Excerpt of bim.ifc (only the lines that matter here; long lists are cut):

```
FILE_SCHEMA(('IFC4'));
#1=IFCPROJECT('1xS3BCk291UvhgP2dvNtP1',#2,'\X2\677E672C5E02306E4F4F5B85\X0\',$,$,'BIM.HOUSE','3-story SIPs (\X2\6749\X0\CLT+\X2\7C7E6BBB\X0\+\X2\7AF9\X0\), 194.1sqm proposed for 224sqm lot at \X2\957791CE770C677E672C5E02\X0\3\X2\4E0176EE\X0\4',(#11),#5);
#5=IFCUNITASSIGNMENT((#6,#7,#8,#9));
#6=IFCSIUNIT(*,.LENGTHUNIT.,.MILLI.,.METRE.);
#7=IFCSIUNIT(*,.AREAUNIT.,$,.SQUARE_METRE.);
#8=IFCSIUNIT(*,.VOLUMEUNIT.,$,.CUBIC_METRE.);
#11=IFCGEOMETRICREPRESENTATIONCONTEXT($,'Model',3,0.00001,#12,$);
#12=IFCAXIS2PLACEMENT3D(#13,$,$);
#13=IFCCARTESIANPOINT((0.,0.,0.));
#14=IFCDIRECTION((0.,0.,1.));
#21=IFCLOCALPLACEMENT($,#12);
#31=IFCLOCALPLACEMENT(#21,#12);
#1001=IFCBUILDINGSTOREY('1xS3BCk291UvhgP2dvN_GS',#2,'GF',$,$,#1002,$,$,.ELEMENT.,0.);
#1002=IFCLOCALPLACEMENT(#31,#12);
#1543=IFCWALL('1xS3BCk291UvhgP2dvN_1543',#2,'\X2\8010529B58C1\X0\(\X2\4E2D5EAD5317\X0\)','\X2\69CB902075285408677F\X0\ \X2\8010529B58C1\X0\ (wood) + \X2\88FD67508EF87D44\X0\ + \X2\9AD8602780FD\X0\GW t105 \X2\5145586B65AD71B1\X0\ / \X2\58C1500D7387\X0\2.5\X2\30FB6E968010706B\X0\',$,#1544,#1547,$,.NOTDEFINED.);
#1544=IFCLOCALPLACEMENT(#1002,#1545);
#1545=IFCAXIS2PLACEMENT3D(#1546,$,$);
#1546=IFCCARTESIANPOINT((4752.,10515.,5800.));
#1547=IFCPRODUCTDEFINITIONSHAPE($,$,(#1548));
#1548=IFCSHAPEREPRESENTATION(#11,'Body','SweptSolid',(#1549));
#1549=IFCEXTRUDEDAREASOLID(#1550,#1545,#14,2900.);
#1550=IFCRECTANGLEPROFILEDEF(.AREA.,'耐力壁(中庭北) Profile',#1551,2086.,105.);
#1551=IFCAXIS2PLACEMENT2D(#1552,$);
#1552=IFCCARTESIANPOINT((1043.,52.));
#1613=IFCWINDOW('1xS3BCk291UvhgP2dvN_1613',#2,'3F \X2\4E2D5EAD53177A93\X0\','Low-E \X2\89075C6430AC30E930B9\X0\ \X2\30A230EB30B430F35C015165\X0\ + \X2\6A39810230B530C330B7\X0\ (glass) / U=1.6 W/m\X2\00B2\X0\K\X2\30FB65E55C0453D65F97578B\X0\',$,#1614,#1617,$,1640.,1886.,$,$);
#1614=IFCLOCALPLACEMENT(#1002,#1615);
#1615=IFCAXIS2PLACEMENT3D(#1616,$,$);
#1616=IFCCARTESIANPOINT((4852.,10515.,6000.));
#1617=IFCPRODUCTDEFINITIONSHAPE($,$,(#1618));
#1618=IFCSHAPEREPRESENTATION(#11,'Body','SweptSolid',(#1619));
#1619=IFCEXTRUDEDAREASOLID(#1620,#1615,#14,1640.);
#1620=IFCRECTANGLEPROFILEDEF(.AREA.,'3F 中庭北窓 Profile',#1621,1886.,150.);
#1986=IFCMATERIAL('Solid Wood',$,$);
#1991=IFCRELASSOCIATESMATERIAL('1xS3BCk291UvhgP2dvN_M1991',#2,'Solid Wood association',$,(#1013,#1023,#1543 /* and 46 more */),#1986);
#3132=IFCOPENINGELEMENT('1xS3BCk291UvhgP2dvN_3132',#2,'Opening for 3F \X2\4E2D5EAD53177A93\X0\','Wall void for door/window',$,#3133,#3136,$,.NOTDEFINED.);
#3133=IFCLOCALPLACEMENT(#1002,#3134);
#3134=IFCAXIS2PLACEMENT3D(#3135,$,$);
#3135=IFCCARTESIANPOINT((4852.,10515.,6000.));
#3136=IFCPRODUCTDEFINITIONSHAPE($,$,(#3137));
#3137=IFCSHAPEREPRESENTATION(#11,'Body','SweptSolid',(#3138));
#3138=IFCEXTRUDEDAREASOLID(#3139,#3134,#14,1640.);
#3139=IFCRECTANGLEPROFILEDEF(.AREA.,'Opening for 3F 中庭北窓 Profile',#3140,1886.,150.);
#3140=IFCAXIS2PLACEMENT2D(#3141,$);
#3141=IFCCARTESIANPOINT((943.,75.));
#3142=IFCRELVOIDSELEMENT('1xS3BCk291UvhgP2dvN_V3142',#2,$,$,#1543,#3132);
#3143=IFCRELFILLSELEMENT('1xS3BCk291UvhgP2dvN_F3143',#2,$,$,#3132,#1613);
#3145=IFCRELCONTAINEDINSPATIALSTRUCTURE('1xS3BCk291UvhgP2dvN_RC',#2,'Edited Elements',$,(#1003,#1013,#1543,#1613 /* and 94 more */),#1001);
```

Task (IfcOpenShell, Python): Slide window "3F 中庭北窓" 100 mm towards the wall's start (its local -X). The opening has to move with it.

```python
import ifcopenshell
import ifcopenshell.api.geometry
import ifcopenshell.util.placement

model = ifcopenshell.open("bim.ifc")

window = model.by_guid("1xS3BCk291UvhgP2dvN_1613")
opening = window.FillsVoids[0].RelatingOpeningElement
wall = opening.VoidsElements[0].RelatingBuildingElement

wall_matrix = ifcopenshell.util.placement.get_local_placement(wall.ObjectPlacement)
shift = wall_matrix[:3, 0] * -100.0
before = ifcopenshell.util.placement.get_local_placement(window.ObjectPlacement)[:3, 3].copy()

# The window is not placed relative to its opening, so move both.
for product in (opening, window):
    matrix = ifcopenshell.util.placement.get_local_placement(product.ObjectPlacement)
    matrix[:3, 3] += shift
    ifcopenshell.api.geometry.edit_object_placement(model, product=product, matrix=matrix, is_si=False)

after = ifcopenshell.util.placement.get_local_placement(window.ObjectPlacement)[:3, 3]
print("window moved by", (after - before).round(3) + 0.0)

model.write("bim_edited.ifc")
```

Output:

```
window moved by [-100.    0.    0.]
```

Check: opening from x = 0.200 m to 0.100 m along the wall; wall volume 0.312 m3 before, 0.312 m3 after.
